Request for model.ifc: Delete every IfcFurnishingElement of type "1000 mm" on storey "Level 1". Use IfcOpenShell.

First a look at what the model holds.

```python
import ifcopenshell
import ifcopenshell.util.element

model = ifcopenshell.open("model.ifc")
print(model.schema)
storey = next(s for s in model.by_type("IfcBuildingStorey") if s.Name == "Level 1")
furniture = [e for e in ifcopenshell.util.element.get_decomposition(storey) if e.is_a("IfcFurnishingElement")]
seen = {}
for e in furniture:
    element_type = ifcopenshell.util.element.get_type(e)
    name = element_type.Name if element_type not in (None, e) else None
    seen[name] = seen.get(name, 0) + 1
for name, count in sorted(seen.items(), key=str):
    print(count, "x", name)
```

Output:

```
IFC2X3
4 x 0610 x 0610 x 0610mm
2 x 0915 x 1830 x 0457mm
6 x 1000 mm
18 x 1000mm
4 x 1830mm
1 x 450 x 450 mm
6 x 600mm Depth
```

```python
import ifcopenshell
import ifcopenshell.api.root
import ifcopenshell.util.element

model = ifcopenshell.open("model.ifc")

storey = next(s for s in model.by_type("IfcBuildingStorey") if s.Name == "Level 1")
furniture = [e for e in ifcopenshell.util.element.get_decomposition(storey) if e.is_a("IfcFurnishingElement")]
targets = [e for e in furniture if (t := ifcopenshell.util.element.get_type(e)) not in (None, e) and t.Name == "1000 mm"]

for e in targets:
    ifcopenshell.api.root.remove_product(model, product=e)
print(len(targets), "removed")

model.write("model_updated.ifc")
```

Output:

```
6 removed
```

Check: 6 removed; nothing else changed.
